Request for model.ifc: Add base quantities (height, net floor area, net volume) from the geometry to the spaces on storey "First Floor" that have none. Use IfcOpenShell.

First a look at what the model holds.

```python
import ifcopenshell
import ifcopenshell.util.element
import ifcopenshell.util.unit

model = ifcopenshell.open("model.ifc")
print(model.schema)
for unit_type in ("LENGTHUNIT", "AREAUNIT", "VOLUMEUNIT"):
    print(unit_type, ifcopenshell.util.unit.calculate_unit_scale(model, unit_type))
storey = next(s for s in model.by_type("IfcBuildingStorey") if s.Name == "First Floor")
spaces = [e for e in ifcopenshell.util.element.get_decomposition(storey) if e.is_a("IfcSpace")]
for e in sorted(spaces, key=lambda e: e.id()):
    print(e.id(), e.is_a(), e.Name, list(ifcopenshell.util.element.get_psets(e, qtos_only=True)), sep=" | ")
```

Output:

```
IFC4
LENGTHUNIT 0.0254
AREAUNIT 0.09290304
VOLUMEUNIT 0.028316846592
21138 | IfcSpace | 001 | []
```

```python
import ifcopenshell
import ifcopenshell.api.pset
import ifcopenshell.geom
import ifcopenshell.util.element
import ifcopenshell.util.shape
import ifcopenshell.util.unit

model = ifcopenshell.open("model.ifc")
unit_scale = ifcopenshell.util.unit.calculate_unit_scale(model)
area_scale = ifcopenshell.util.unit.calculate_unit_scale(model, "AREAUNIT")
volume_scale = ifcopenshell.util.unit.calculate_unit_scale(model, "VOLUMEUNIT")
settings = ifcopenshell.geom.settings()

storey = next(s for s in model.by_type("IfcBuildingStorey") if s.Name == "First Floor")
spaces = [e for e in ifcopenshell.util.element.get_decomposition(storey) if e.is_a("IfcSpace")]

for e in sorted(spaces, key=lambda e: e.id()):
    if ifcopenshell.util.element.get_psets(e, qtos_only=True, should_inherit=False):
        continue
    # Geometry comes back in metres, in the element's own axes.
    shape = ifcopenshell.geom.create_shape(settings, e)
    values = {
        "Height": ifcopenshell.util.shape.get_z(shape.geometry) / unit_scale,
        "NetFloorArea": ifcopenshell.util.shape.get_footprint_area(shape.geometry) / area_scale,
        "NetVolume": ifcopenshell.util.shape.get_volume(shape.geometry) / volume_scale,
    }
    qto = ifcopenshell.api.pset.add_qto(model, product=e, name="Qto_SpaceBaseQuantities")
    ifcopenshell.api.pset.edit_qto(model, qto=qto, properties=values)
    print(e.id(), {k: round(v, 3) for k, v in values.items()})

model.write("model_rev.ifc")
```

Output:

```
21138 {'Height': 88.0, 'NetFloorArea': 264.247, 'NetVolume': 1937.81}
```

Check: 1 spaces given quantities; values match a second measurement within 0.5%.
